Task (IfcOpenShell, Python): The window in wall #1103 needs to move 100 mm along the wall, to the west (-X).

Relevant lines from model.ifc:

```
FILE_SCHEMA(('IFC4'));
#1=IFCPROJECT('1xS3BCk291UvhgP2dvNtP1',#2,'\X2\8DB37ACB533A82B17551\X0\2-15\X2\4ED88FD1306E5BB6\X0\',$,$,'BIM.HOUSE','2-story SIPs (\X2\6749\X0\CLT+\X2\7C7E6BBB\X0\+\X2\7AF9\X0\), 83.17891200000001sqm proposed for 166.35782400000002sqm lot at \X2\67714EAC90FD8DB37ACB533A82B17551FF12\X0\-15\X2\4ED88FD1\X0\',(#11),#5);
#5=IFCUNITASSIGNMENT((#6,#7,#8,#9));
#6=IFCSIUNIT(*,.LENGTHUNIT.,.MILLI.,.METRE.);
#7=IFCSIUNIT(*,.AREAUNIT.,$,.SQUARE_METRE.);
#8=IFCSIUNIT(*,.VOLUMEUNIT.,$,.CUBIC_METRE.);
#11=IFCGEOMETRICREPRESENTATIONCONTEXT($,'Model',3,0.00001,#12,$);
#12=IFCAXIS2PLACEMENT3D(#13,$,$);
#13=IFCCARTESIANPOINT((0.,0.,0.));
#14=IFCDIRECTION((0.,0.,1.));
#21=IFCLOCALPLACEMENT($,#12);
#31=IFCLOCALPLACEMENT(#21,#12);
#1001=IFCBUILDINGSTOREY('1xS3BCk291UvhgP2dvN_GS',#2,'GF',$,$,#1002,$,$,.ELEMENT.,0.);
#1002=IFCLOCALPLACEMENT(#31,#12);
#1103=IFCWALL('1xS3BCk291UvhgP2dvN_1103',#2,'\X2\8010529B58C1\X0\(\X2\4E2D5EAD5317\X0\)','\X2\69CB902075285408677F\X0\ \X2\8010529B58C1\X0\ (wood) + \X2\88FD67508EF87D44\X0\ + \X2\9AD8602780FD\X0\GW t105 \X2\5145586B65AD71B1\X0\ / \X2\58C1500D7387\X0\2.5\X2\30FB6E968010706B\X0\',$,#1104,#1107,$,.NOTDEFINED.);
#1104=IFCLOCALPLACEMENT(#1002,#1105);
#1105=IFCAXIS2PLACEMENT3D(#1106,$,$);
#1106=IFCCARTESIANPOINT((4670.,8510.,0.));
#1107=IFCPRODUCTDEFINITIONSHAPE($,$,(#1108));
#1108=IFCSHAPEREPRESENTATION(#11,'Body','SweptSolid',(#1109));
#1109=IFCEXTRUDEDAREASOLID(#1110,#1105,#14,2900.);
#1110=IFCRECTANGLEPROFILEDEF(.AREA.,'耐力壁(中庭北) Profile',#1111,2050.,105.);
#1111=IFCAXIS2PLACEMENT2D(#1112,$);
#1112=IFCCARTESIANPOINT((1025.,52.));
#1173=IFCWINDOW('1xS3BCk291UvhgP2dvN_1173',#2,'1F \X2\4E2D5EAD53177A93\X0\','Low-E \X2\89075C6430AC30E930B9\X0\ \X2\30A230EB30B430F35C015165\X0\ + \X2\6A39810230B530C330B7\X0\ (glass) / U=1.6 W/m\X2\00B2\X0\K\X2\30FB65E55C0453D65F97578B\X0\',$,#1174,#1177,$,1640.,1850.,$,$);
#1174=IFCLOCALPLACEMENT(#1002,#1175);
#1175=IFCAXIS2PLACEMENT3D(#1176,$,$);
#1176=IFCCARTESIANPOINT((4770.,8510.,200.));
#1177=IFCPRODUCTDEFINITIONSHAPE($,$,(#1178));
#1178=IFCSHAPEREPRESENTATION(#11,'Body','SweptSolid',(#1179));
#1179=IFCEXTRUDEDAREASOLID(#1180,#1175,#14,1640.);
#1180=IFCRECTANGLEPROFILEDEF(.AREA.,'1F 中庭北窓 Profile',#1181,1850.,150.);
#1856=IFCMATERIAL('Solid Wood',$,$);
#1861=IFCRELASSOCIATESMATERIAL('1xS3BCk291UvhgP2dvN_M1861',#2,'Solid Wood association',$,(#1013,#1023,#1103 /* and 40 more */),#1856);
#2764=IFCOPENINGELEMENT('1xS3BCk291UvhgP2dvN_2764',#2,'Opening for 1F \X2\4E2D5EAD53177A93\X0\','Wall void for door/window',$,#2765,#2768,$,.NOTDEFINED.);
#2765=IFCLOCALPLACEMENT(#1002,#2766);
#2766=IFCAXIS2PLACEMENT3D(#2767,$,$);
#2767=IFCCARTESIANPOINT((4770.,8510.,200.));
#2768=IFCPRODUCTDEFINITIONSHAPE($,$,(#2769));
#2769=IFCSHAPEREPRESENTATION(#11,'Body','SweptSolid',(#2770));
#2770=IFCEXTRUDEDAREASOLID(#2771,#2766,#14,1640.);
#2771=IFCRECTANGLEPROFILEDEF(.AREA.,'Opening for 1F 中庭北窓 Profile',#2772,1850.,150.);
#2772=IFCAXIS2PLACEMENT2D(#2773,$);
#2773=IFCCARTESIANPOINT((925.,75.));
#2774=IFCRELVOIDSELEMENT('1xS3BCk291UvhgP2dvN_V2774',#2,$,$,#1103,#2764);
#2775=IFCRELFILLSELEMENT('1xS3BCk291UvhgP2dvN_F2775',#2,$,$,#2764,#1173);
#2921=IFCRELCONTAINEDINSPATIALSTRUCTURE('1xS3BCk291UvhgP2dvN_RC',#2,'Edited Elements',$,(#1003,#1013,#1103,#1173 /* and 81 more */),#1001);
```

```python
import ifcopenshell
import ifcopenshell.api.geometry
import ifcopenshell.util.placement
import ifcopenshell.util.unit

model = ifcopenshell.open("model.ifc")
unit_scale = ifcopenshell.util.unit.calculate_unit_scale(model)

window = model.by_guid("1xS3BCk291UvhgP2dvN_1173")
opening = window.FillsVoids[0].RelatingOpeningElement
wall = opening.VoidsElements[0].RelatingBuildingElement

wall_matrix = ifcopenshell.util.placement.get_local_placement(wall.ObjectPlacement)
shift = wall_matrix[:3, 0] * -0.1 / unit_scale
before = ifcopenshell.util.placement.get_local_placement(window.ObjectPlacement)[:3, 3].copy()

# The window is not placed relative to its opening, so move both.
for product in (opening, window):
    matrix = ifcopenshell.util.placement.get_local_placement(product.ObjectPlacement)
    matrix[:3, 3] += shift
    ifcopenshell.api.geometry.edit_object_placement(model, product=product, matrix=matrix, is_si=False)

after = ifcopenshell.util.placement.get_local_placement(window.ObjectPlacement)[:3, 3]
print("window moved by", (after - before).round(3) + 0.0)

model.write("model_v2.ifc")
```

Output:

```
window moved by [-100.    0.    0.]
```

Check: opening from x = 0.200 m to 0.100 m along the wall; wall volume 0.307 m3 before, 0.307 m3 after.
